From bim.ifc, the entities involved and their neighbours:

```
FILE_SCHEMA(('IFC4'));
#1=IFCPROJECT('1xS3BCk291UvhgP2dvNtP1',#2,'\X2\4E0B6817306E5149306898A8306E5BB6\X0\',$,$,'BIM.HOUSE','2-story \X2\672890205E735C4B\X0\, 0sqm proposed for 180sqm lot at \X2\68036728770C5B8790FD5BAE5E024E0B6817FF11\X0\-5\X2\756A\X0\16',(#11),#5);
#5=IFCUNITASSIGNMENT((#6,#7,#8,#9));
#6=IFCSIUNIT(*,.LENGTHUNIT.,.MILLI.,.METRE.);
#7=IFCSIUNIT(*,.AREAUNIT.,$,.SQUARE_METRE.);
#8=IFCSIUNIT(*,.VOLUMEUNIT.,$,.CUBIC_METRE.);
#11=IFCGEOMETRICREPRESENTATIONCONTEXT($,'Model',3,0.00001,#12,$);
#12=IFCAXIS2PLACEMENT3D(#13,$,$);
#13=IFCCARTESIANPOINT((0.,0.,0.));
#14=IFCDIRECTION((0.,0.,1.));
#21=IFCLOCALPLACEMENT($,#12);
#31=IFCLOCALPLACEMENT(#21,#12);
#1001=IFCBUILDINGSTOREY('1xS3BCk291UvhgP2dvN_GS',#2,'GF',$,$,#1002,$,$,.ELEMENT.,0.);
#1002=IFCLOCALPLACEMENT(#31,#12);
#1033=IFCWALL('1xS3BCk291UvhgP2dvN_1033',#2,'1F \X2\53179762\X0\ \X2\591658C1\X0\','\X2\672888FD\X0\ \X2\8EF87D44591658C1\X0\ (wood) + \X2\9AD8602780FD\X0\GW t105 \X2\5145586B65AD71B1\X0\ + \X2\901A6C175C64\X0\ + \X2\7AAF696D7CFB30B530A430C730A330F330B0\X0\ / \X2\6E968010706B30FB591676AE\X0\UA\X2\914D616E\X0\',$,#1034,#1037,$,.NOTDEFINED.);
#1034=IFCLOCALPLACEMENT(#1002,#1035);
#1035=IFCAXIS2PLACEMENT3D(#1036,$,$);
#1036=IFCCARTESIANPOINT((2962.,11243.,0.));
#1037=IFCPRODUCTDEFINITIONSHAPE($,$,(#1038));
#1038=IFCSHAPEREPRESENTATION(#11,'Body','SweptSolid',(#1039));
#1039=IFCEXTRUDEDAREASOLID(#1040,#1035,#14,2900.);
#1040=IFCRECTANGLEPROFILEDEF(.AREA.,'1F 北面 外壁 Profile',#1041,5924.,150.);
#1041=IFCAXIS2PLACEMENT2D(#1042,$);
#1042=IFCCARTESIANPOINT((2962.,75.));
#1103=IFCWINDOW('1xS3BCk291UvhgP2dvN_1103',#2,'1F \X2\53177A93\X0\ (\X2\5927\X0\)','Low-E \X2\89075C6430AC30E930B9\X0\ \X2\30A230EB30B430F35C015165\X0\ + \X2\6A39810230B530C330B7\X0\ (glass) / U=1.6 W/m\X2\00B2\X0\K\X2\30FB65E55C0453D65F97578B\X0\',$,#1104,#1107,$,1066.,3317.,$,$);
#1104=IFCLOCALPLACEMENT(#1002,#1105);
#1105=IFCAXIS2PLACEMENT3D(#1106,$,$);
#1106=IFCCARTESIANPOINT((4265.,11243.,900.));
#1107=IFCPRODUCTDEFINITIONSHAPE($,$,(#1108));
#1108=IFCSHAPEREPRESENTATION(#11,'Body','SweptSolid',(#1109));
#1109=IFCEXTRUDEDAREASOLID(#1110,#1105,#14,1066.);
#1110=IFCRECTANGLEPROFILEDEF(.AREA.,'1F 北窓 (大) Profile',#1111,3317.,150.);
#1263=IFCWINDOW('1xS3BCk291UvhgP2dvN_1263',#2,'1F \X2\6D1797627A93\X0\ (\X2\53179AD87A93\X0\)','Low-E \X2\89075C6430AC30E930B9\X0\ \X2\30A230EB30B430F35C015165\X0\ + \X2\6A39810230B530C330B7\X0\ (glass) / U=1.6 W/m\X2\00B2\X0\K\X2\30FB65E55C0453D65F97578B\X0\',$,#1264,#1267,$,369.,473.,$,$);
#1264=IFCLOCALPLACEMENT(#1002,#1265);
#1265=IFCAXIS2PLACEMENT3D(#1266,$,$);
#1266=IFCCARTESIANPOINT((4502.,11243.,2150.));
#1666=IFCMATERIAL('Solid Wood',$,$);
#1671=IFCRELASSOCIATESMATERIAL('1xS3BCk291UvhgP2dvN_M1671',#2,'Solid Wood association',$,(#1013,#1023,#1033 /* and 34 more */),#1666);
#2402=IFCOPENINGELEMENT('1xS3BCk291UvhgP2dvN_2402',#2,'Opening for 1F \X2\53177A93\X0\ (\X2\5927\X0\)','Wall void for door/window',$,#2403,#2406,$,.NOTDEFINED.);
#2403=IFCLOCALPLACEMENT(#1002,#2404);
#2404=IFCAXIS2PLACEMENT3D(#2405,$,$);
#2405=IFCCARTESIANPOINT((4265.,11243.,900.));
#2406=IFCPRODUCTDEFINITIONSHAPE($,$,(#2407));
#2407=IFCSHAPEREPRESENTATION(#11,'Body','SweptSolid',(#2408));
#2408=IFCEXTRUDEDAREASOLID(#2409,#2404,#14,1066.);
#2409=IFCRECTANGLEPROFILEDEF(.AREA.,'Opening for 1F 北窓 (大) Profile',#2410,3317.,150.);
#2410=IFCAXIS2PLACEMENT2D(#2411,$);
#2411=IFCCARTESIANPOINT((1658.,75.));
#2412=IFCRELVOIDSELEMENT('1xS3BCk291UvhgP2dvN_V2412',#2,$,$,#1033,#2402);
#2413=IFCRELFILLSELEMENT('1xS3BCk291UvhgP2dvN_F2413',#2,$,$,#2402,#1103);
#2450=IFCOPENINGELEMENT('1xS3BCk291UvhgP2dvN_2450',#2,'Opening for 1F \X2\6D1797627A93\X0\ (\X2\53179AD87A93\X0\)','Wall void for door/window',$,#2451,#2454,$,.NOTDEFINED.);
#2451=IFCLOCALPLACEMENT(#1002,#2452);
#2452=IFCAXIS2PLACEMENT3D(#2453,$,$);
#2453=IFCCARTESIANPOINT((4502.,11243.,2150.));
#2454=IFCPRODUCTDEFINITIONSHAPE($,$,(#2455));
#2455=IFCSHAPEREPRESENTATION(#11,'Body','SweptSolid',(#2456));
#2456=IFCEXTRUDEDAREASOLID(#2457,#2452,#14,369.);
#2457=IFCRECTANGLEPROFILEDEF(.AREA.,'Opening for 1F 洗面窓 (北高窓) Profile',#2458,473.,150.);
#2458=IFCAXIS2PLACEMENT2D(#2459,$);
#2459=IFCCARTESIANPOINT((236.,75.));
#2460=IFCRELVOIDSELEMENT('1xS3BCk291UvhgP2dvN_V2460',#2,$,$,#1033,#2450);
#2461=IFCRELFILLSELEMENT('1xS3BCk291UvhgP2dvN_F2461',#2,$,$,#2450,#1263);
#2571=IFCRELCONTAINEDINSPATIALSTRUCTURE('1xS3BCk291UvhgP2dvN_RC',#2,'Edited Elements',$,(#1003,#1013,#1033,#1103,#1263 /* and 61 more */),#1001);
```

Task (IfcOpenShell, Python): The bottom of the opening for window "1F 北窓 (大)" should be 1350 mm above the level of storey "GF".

```python
import numpy as np
import ifcopenshell
import ifcopenshell.api.geometry
import ifcopenshell.geom
import ifcopenshell.util.element
import ifcopenshell.util.placement
import ifcopenshell.util.shape
import ifcopenshell.util.unit

model = ifcopenshell.open("bim.ifc")
unit_scale = ifcopenshell.util.unit.calculate_unit_scale(model)

window = model.by_guid("1xS3BCk291UvhgP2dvN_1103")
opening = window.FillsVoids[0].RelatingOpeningElement
storey = ifcopenshell.util.element.get_container(window, ifc_class="IfcBuildingStorey")
level = ifcopenshell.util.placement.get_local_placement(storey.ObjectPlacement)[2, 3]

# The opening's origin need not be at the sill, so measure its lowest point.
shape = ifcopenshell.geom.create_shape(ifcopenshell.geom.settings(), opening)
bottom = ifcopenshell.util.shape.get_shape_bottom_elevation(shape, shape.geometry) / unit_scale
dz = level + 1350.0 - bottom

shift = np.array([0.0, 0.0, dz])
# The window is not placed relative to its opening, so move both.
for product in (opening, window):
    matrix = ifcopenshell.util.placement.get_local_placement(product.ObjectPlacement)
    matrix[:3, 3] += shift
    ifcopenshell.api.geometry.edit_object_placement(model, product=product, matrix=matrix, is_si=False)

print(f"moved by {dz * unit_scale:+.3f} m")

model.write("bim_rev.ifc")
```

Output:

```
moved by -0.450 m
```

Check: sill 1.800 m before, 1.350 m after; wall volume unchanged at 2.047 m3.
